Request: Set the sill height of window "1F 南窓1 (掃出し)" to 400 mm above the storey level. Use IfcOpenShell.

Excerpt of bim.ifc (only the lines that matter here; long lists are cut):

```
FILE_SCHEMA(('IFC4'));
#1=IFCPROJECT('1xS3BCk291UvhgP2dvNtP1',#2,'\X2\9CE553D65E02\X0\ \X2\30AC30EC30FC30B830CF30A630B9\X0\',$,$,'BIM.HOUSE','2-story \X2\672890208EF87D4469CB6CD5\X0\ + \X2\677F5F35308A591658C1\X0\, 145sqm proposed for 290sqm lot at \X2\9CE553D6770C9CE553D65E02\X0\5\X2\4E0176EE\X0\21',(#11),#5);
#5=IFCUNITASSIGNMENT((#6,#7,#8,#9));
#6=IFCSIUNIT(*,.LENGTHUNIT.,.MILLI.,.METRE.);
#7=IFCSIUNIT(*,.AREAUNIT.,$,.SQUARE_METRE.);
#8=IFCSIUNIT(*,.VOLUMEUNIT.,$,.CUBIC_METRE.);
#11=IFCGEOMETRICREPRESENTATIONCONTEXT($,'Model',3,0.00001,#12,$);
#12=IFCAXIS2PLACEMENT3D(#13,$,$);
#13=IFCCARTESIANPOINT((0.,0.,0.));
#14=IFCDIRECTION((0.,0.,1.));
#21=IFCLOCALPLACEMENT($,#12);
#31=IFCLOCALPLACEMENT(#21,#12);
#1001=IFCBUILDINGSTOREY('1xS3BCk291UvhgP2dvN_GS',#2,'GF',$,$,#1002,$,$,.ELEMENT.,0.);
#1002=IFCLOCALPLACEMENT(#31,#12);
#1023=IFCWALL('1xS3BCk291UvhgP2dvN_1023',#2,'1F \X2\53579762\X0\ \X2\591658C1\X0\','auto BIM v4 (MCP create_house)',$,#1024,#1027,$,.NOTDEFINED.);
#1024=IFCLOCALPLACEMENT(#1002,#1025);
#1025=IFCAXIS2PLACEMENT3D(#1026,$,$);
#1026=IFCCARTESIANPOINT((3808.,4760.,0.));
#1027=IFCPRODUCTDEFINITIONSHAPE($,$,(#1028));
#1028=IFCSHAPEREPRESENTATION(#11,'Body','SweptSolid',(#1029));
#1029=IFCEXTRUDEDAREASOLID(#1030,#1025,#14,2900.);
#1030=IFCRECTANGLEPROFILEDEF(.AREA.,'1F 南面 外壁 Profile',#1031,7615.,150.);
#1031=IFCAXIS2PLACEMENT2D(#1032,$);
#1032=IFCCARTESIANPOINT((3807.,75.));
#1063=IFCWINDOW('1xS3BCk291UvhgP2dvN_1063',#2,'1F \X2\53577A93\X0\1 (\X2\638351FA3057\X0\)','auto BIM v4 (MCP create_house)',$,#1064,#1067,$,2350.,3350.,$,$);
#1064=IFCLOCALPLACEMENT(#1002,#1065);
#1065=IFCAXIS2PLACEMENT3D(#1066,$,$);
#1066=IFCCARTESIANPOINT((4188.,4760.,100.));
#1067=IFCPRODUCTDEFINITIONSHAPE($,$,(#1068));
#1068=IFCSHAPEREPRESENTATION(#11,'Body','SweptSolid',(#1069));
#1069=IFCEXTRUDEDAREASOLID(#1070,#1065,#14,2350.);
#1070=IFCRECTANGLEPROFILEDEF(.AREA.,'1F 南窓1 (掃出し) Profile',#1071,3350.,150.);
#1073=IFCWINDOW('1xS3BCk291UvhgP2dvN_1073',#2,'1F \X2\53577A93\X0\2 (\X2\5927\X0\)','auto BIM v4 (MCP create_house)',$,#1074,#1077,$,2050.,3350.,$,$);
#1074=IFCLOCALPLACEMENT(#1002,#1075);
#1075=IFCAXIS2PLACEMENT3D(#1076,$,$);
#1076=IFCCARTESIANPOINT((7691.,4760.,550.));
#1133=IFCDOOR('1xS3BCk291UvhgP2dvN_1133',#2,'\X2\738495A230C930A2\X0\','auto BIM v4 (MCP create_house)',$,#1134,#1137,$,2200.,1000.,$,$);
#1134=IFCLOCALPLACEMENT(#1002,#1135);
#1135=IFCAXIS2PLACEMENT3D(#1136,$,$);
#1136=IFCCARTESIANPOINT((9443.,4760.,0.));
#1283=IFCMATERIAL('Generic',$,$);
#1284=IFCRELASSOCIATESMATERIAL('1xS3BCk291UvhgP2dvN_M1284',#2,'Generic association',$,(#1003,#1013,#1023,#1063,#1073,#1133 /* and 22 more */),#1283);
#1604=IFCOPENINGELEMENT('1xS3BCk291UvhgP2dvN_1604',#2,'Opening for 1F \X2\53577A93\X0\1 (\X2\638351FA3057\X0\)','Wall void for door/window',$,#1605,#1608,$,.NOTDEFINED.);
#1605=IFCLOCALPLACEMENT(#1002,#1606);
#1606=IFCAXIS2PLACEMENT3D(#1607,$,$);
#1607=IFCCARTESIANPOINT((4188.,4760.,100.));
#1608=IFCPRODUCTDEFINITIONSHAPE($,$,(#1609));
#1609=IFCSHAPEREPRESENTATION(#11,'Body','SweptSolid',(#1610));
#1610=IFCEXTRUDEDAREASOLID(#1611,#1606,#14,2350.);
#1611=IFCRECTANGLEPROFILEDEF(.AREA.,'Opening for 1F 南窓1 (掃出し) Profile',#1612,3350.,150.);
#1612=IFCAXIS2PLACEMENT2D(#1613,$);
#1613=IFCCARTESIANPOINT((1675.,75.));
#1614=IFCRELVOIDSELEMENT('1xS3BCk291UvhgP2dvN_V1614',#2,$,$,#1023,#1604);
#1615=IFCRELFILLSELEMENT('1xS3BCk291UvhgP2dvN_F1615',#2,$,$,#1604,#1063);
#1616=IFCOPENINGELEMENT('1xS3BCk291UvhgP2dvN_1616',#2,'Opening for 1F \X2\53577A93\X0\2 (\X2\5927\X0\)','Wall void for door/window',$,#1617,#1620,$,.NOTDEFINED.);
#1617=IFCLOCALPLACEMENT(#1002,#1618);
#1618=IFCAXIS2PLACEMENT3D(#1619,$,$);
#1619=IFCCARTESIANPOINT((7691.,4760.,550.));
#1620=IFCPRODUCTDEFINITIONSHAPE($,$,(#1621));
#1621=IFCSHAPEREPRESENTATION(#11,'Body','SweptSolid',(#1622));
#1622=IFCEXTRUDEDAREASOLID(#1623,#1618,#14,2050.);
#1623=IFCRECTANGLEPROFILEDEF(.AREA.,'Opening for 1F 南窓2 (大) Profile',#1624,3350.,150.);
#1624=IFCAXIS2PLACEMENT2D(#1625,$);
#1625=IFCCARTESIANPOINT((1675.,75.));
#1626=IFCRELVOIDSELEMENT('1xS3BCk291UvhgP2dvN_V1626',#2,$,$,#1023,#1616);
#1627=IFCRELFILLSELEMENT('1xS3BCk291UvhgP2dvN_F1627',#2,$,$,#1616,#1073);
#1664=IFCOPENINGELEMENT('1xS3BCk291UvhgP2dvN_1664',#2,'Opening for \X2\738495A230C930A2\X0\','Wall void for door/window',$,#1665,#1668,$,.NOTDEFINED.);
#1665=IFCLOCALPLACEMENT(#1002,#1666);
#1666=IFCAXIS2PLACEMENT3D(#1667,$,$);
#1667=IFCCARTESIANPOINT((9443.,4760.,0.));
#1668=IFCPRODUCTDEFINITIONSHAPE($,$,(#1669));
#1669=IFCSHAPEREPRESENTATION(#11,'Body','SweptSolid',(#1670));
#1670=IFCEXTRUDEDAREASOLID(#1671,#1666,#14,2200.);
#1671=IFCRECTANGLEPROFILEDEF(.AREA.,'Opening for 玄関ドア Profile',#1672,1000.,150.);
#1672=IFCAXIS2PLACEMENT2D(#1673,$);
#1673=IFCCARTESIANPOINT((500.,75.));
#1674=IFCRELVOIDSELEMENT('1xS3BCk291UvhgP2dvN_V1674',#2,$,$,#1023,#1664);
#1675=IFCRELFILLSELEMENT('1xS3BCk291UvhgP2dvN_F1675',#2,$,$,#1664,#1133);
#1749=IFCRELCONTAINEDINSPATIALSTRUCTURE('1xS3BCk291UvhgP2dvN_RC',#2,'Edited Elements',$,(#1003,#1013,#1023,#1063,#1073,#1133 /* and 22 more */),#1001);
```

```python
import numpy as np
import ifcopenshell
import ifcopenshell.api.geometry
import ifcopenshell.geom
import ifcopenshell.util.element
import ifcopenshell.util.placement
import ifcopenshell.util.shape
import ifcopenshell.util.unit

model = ifcopenshell.open("bim.ifc")
unit_scale = ifcopenshell.util.unit.calculate_unit_scale(model)

window = model.by_guid("1xS3BCk291UvhgP2dvN_1063")
opening = window.FillsVoids[0].RelatingOpeningElement
storey = ifcopenshell.util.element.get_container(window, ifc_class="IfcBuildingStorey")
level = ifcopenshell.util.placement.get_local_placement(storey.ObjectPlacement)[2, 3]

# The opening's origin need not be at the sill, so measure its lowest point.
shape = ifcopenshell.geom.create_shape(ifcopenshell.geom.settings(), opening)
bottom = ifcopenshell.util.shape.get_shape_bottom_elevation(shape, shape.geometry) / unit_scale
dz = level + 400.0 - bottom

shift = np.array([0.0, 0.0, dz])
# The window is not placed relative to its opening, so move both.
for product in (opening, window):
    matrix = ifcopenshell.util.placement.get_local_placement(product.ObjectPlacement)
    matrix[:3, 3] += shift
    ifcopenshell.api.geometry.edit_object_placement(model, product=product, matrix=matrix, is_si=False)

print(f"moved by {dz * unit_scale:+.3f} m")

model.write("bim_rev.ifc")
```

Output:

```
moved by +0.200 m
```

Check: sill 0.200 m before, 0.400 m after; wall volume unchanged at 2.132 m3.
